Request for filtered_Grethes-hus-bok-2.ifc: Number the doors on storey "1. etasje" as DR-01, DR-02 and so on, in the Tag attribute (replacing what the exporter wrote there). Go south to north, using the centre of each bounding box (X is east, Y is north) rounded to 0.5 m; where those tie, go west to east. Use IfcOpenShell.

First a look at what the model holds.

```python
import ifcopenshell
import ifcopenshell.util.element
import ifcopenshell.util.placement

model = ifcopenshell.open("filtered_Grethes-hus-bok-2.ifc")
print(model.schema)
storey = next(s for s in model.by_type("IfcBuildingStorey") if s.Name == "1. etasje")
doors = [e for e in ifcopenshell.util.element.get_decomposition(storey) if e.is_a("IfcDoor")]
for e in sorted(doors, key=lambda e: e.id()):
    origin = ifcopenshell.util.placement.get_local_placement(e.ObjectPlacement)[:3, 3]
    print(e.id(), e.Tag, e.Name, origin.round(2) + 0.0, sep=" | ")
```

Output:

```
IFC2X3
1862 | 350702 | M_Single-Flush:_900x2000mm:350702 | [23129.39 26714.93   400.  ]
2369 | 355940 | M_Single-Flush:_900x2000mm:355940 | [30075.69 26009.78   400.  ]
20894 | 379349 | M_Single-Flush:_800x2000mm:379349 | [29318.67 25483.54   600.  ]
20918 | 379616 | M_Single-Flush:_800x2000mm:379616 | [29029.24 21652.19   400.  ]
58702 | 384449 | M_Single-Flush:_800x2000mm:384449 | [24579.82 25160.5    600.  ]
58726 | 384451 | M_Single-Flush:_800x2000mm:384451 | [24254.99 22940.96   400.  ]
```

```python
import ifcopenshell
import ifcopenshell.geom
import ifcopenshell.util.element
import ifcopenshell.util.shape

model = ifcopenshell.open("filtered_Grethes-hus-bok-2.ifc")
settings = ifcopenshell.geom.settings()
settings.set("use-world-coords", True)


def centre(element):
    shape = ifcopenshell.geom.create_shape(settings, element)
    return ifcopenshell.util.shape.get_bbox_centroid(shape.geometry)


storey = next(s for s in model.by_type("IfcBuildingStorey") if s.Name == "1. etasje")
doors = [e for e in ifcopenshell.util.element.get_decomposition(storey) if e.is_a("IfcDoor")]

# Insertion points can sit at a corner or the storey origin, so sort by the geometry (in metres).
centres = {e: centre(e) for e in doors}
doors.sort(key=lambda e: (round(centres[e][1] / 0.5), centres[e][0]))

for i, e in enumerate(doors, start=1):
    number = f"DR-{i:02d}"
    e.Tag = number
    print(e.id(), number)

model.write("filtered_Grethes-hus-bok-2-out.ifc")
```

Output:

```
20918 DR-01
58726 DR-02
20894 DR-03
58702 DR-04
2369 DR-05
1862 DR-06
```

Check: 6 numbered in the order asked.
